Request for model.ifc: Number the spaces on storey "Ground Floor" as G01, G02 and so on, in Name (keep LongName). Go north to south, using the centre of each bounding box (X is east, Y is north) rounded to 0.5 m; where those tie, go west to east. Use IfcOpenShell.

First a look at what the model holds.

```python
import ifcopenshell
import ifcopenshell.util.element
import ifcopenshell.util.placement

model = ifcopenshell.open("model.ifc")
print(model.schema)
storey = next(s for s in model.by_type("IfcBuildingStorey") if s.Name == "Ground Floor")
spaces = [e for e in ifcopenshell.util.element.get_decomposition(storey) if e.is_a("IfcSpace")]
for e in sorted(spaces, key=lambda e: e.id()):
    origin = ifcopenshell.util.placement.get_local_placement(e.ObjectPlacement)[:3, 3]
    print(e.id(), e.Name, e.LongName, origin.round(2) + 0.0, sep=" | ")
```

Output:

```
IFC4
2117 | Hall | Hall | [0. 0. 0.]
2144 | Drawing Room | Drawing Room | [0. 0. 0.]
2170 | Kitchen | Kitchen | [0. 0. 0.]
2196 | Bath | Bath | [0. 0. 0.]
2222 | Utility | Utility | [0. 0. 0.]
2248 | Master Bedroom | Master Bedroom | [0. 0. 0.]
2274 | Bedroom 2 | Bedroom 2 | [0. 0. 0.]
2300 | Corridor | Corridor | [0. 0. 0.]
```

```python
import ifcopenshell
import ifcopenshell.geom
import ifcopenshell.util.element
import ifcopenshell.util.shape

model = ifcopenshell.open("model.ifc")
settings = ifcopenshell.geom.settings()
settings.set("use-world-coords", True)


def centre(element):
    shape = ifcopenshell.geom.create_shape(settings, element)
    return ifcopenshell.util.shape.get_bbox_centroid(shape.geometry)


storey = next(s for s in model.by_type("IfcBuildingStorey") if s.Name == "Ground Floor")
spaces = [e for e in ifcopenshell.util.element.get_decomposition(storey) if e.is_a("IfcSpace")]

# Insertion points can sit at a corner or the storey origin, so sort by the geometry (in metres).
centres = {e: centre(e) for e in spaces}
spaces.sort(key=lambda e: (-round(centres[e][1] / 0.5), centres[e][0]))

for i, e in enumerate(spaces, start=1):
    number = f"G{i:02d}"
    e.Name = number
    print(e.id(), number)

model.write("model-out.ifc")
```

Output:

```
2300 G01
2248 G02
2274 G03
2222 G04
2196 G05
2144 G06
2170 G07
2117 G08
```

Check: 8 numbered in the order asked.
